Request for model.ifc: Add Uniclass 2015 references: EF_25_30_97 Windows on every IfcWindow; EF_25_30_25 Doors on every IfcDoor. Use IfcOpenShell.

First a look at what the model holds.

```python
import ifcopenshell

model = ifcopenshell.open("model.ifc")
print(model.schema)
print("classifications:", [c.Name for c in model.by_type("IfcClassification")])
for ifc_class in ("IfcDoor", "IfcRoof", "IfcStair", "IfcWall", "IfcWindow"):
    print(ifc_class, len(model.by_type(ifc_class)))
```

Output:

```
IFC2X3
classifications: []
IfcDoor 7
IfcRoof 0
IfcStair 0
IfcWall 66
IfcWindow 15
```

```python
import ifcopenshell
import ifcopenshell.api.classification

model = ifcopenshell.open("model.ifc")

# IFC2X3 requires Source and Edition and has no link from the project to the system.
system = model.create_entity("IfcClassification", Source="NBS", Edition="2015", Name="Uniclass 2015")

codes = {
    "IfcWindow": ("EF_25_30_97", "Windows"),
    "IfcDoor": ("EF_25_30_25", "Doors"),
}
for ifc_class, (code, name) in codes.items():
    products = model.by_type(ifc_class)
    ifcopenshell.api.classification.add_reference(
        model, products=products, classification=system, identification=code, name=name
    )
    print(code, len(products))

model.write("model_rev.ifc")
```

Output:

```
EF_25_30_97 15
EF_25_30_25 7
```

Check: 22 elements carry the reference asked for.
